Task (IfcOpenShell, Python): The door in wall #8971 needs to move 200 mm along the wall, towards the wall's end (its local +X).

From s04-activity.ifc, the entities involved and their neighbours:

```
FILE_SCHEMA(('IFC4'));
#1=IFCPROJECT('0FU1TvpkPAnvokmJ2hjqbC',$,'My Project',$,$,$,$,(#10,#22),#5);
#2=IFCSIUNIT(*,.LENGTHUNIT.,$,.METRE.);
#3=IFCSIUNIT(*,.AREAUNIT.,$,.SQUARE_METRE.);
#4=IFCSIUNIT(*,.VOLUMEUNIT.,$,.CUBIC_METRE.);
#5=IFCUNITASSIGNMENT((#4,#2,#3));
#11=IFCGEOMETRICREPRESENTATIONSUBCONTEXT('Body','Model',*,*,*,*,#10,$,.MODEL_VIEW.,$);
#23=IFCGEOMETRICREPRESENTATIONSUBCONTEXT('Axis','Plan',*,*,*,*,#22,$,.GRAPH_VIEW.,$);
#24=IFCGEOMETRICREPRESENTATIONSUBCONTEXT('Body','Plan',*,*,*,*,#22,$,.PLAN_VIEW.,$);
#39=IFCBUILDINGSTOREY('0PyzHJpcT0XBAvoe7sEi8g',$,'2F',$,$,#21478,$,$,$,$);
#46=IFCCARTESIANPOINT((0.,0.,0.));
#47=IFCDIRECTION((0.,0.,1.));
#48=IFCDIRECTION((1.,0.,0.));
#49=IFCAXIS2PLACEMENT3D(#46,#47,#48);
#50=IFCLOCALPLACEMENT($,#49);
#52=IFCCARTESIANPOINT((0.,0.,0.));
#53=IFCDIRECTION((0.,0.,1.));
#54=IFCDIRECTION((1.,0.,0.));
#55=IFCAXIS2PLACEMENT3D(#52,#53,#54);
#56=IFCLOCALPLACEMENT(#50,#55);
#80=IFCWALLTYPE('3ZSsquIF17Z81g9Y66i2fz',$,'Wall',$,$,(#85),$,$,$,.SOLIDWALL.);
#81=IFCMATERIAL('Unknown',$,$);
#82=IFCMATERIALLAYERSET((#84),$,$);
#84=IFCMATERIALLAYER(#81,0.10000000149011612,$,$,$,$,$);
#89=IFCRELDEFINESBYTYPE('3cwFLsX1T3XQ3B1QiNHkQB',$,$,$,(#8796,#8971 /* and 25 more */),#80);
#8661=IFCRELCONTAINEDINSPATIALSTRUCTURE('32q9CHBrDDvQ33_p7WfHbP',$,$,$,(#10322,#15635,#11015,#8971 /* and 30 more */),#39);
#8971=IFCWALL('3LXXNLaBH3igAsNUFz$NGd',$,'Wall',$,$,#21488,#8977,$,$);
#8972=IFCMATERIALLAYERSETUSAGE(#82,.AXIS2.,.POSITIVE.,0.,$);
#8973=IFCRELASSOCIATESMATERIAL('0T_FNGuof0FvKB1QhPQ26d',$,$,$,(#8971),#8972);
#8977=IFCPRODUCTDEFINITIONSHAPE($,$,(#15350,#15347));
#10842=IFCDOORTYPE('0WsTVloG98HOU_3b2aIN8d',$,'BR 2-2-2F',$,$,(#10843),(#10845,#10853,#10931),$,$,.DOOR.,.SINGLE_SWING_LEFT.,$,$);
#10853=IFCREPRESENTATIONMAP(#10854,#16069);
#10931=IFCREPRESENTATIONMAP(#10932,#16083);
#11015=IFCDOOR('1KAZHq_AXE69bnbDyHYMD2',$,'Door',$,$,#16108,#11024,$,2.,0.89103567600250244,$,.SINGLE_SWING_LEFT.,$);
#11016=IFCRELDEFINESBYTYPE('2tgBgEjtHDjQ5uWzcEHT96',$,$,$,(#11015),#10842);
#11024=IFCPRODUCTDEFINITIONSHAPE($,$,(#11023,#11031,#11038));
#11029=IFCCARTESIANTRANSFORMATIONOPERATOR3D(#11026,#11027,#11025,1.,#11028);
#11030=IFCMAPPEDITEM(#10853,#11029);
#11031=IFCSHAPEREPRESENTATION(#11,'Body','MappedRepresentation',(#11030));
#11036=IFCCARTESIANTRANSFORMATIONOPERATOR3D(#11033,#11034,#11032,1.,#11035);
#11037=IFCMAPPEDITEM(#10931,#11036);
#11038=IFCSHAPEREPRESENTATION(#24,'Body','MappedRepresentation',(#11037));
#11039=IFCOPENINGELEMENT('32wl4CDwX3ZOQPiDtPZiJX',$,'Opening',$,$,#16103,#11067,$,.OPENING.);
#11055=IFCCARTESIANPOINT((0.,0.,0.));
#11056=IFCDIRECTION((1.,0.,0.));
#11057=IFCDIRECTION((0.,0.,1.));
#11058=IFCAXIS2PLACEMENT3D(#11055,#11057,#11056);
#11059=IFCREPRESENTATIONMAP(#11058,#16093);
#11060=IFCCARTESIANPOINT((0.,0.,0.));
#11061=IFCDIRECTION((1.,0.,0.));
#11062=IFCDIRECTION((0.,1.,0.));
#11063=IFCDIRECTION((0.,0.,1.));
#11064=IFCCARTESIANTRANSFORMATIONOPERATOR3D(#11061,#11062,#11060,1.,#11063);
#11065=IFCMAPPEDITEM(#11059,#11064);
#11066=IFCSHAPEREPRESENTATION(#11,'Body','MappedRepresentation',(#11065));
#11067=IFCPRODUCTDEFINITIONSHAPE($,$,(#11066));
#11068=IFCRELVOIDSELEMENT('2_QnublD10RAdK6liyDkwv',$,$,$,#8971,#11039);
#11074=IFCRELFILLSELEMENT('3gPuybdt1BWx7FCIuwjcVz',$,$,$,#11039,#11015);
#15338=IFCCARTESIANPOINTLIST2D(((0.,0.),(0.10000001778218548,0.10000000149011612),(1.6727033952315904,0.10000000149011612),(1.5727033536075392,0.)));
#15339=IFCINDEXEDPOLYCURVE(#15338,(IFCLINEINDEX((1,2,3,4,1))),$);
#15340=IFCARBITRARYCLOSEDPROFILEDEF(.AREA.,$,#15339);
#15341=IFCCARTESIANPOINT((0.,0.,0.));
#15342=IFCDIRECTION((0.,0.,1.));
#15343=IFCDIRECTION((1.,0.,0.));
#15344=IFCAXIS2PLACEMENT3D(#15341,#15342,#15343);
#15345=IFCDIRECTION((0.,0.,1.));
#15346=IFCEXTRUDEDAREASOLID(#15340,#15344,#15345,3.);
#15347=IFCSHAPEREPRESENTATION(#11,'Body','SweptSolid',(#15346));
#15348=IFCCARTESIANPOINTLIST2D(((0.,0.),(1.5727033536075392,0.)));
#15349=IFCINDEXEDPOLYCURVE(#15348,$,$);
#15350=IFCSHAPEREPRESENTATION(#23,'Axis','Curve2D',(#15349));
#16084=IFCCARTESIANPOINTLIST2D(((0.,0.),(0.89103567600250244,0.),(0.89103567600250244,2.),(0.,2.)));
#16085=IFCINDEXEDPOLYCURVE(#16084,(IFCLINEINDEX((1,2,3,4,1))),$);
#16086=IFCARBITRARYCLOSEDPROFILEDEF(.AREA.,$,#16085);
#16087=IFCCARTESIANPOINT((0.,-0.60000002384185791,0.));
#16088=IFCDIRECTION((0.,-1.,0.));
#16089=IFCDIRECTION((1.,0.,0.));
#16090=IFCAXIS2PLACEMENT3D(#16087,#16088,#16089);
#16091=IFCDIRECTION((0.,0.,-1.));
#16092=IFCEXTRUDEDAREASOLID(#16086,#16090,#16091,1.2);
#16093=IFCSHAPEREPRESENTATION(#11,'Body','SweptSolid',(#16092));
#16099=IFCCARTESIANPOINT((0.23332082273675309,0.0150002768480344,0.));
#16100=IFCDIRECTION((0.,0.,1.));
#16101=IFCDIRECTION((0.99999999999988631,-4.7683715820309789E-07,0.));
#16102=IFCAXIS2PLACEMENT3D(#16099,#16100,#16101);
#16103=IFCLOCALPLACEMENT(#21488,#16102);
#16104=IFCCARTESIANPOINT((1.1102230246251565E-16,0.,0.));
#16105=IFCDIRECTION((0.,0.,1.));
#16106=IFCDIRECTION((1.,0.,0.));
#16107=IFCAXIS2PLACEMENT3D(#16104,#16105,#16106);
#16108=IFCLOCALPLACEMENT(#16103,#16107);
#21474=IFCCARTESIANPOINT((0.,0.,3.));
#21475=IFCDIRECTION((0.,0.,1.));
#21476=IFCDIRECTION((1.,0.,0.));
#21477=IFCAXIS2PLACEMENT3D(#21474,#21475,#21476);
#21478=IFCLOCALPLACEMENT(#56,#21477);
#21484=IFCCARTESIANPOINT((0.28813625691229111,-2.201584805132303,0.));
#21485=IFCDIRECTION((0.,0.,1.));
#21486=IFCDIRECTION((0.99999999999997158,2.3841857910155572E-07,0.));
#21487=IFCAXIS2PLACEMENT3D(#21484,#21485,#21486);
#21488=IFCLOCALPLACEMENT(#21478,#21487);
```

```python
import ifcopenshell
import ifcopenshell.api.geometry
import ifcopenshell.util.placement
import ifcopenshell.util.unit

model = ifcopenshell.open("s04-activity.ifc")
unit_scale = ifcopenshell.util.unit.calculate_unit_scale(model)

door = model.by_guid("1KAZHq_AXE69bnbDyHYMD2")
opening = door.FillsVoids[0].RelatingOpeningElement
wall = opening.VoidsElements[0].RelatingBuildingElement

wall_matrix = ifcopenshell.util.placement.get_local_placement(wall.ObjectPlacement)
shift = wall_matrix[:3, 0] * 0.2 / unit_scale
before = ifcopenshell.util.placement.get_local_placement(door.ObjectPlacement)[:3, 3].copy()

# The door is placed relative to its opening, so it follows when the opening moves.
matrix = ifcopenshell.util.placement.get_local_placement(opening.ObjectPlacement)
matrix[:3, 3] += shift
ifcopenshell.api.geometry.edit_object_placement(
    model, product=opening, matrix=matrix, is_si=False, should_transform_children=True
)

after = ifcopenshell.util.placement.get_local_placement(door.ObjectPlacement)[:3, 3]
print("door moved by", (after - before).round(3) + 0.0)

model.write("s04-activity_updated.ifc")
```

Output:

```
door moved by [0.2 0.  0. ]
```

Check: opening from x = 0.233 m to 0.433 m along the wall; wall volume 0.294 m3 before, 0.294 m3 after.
